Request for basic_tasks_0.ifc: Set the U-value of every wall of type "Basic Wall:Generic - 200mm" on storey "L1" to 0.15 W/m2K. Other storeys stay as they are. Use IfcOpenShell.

First a look at what the model holds.

```python
import ifcopenshell
import ifcopenshell.util.element

model = ifcopenshell.open("basic_tasks_0.ifc")
print(model.schema)
storey = next(s for s in model.by_type("IfcBuildingStorey") if s.Name == "L1")
walls = [e for e in ifcopenshell.util.element.get_decomposition(storey) if e.is_a("IfcWall")]
seen = {}
for e in walls:
    element_type = ifcopenshell.util.element.get_type(e)
    key = (element_type.Name if element_type != e and element_type else None, ifcopenshell.util.element.get_pset(e, "Pset_WallCommon", "ThermalTransmittance"))
    seen[key] = seen.get(key, 0) + 1
for (name, value), count in sorted(seen.items(), key=str):
    print(count, "x", name, "|", value)
```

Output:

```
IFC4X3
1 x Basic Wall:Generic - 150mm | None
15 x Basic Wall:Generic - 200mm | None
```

```python
import ifcopenshell
import ifcopenshell.api.pset
import ifcopenshell.util.element

model = ifcopenshell.open("basic_tasks_0.ifc")

storey = next(s for s in model.by_type("IfcBuildingStorey") if s.Name == "L1")
walls = [e for e in ifcopenshell.util.element.get_decomposition(storey) if e.is_a("IfcWall")]

count = 0
for e in walls:
    element_type = ifcopenshell.util.element.get_type(e)
    if element_type in (None, e) or element_type.Name != "Basic Wall:Generic - 200mm":
        continue
    # add_pset returns the element's existing set when there is one.
    pset = ifcopenshell.api.pset.add_pset(model, product=e, name="Pset_WallCommon")
    ifcopenshell.api.pset.edit_pset(model, pset=pset, properties={"ThermalTransmittance": 0.15})
    count += 1

print(count, "walls updated")

model.write("basic_tasks_0_rev.ifc")
```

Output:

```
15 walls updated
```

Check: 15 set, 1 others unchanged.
